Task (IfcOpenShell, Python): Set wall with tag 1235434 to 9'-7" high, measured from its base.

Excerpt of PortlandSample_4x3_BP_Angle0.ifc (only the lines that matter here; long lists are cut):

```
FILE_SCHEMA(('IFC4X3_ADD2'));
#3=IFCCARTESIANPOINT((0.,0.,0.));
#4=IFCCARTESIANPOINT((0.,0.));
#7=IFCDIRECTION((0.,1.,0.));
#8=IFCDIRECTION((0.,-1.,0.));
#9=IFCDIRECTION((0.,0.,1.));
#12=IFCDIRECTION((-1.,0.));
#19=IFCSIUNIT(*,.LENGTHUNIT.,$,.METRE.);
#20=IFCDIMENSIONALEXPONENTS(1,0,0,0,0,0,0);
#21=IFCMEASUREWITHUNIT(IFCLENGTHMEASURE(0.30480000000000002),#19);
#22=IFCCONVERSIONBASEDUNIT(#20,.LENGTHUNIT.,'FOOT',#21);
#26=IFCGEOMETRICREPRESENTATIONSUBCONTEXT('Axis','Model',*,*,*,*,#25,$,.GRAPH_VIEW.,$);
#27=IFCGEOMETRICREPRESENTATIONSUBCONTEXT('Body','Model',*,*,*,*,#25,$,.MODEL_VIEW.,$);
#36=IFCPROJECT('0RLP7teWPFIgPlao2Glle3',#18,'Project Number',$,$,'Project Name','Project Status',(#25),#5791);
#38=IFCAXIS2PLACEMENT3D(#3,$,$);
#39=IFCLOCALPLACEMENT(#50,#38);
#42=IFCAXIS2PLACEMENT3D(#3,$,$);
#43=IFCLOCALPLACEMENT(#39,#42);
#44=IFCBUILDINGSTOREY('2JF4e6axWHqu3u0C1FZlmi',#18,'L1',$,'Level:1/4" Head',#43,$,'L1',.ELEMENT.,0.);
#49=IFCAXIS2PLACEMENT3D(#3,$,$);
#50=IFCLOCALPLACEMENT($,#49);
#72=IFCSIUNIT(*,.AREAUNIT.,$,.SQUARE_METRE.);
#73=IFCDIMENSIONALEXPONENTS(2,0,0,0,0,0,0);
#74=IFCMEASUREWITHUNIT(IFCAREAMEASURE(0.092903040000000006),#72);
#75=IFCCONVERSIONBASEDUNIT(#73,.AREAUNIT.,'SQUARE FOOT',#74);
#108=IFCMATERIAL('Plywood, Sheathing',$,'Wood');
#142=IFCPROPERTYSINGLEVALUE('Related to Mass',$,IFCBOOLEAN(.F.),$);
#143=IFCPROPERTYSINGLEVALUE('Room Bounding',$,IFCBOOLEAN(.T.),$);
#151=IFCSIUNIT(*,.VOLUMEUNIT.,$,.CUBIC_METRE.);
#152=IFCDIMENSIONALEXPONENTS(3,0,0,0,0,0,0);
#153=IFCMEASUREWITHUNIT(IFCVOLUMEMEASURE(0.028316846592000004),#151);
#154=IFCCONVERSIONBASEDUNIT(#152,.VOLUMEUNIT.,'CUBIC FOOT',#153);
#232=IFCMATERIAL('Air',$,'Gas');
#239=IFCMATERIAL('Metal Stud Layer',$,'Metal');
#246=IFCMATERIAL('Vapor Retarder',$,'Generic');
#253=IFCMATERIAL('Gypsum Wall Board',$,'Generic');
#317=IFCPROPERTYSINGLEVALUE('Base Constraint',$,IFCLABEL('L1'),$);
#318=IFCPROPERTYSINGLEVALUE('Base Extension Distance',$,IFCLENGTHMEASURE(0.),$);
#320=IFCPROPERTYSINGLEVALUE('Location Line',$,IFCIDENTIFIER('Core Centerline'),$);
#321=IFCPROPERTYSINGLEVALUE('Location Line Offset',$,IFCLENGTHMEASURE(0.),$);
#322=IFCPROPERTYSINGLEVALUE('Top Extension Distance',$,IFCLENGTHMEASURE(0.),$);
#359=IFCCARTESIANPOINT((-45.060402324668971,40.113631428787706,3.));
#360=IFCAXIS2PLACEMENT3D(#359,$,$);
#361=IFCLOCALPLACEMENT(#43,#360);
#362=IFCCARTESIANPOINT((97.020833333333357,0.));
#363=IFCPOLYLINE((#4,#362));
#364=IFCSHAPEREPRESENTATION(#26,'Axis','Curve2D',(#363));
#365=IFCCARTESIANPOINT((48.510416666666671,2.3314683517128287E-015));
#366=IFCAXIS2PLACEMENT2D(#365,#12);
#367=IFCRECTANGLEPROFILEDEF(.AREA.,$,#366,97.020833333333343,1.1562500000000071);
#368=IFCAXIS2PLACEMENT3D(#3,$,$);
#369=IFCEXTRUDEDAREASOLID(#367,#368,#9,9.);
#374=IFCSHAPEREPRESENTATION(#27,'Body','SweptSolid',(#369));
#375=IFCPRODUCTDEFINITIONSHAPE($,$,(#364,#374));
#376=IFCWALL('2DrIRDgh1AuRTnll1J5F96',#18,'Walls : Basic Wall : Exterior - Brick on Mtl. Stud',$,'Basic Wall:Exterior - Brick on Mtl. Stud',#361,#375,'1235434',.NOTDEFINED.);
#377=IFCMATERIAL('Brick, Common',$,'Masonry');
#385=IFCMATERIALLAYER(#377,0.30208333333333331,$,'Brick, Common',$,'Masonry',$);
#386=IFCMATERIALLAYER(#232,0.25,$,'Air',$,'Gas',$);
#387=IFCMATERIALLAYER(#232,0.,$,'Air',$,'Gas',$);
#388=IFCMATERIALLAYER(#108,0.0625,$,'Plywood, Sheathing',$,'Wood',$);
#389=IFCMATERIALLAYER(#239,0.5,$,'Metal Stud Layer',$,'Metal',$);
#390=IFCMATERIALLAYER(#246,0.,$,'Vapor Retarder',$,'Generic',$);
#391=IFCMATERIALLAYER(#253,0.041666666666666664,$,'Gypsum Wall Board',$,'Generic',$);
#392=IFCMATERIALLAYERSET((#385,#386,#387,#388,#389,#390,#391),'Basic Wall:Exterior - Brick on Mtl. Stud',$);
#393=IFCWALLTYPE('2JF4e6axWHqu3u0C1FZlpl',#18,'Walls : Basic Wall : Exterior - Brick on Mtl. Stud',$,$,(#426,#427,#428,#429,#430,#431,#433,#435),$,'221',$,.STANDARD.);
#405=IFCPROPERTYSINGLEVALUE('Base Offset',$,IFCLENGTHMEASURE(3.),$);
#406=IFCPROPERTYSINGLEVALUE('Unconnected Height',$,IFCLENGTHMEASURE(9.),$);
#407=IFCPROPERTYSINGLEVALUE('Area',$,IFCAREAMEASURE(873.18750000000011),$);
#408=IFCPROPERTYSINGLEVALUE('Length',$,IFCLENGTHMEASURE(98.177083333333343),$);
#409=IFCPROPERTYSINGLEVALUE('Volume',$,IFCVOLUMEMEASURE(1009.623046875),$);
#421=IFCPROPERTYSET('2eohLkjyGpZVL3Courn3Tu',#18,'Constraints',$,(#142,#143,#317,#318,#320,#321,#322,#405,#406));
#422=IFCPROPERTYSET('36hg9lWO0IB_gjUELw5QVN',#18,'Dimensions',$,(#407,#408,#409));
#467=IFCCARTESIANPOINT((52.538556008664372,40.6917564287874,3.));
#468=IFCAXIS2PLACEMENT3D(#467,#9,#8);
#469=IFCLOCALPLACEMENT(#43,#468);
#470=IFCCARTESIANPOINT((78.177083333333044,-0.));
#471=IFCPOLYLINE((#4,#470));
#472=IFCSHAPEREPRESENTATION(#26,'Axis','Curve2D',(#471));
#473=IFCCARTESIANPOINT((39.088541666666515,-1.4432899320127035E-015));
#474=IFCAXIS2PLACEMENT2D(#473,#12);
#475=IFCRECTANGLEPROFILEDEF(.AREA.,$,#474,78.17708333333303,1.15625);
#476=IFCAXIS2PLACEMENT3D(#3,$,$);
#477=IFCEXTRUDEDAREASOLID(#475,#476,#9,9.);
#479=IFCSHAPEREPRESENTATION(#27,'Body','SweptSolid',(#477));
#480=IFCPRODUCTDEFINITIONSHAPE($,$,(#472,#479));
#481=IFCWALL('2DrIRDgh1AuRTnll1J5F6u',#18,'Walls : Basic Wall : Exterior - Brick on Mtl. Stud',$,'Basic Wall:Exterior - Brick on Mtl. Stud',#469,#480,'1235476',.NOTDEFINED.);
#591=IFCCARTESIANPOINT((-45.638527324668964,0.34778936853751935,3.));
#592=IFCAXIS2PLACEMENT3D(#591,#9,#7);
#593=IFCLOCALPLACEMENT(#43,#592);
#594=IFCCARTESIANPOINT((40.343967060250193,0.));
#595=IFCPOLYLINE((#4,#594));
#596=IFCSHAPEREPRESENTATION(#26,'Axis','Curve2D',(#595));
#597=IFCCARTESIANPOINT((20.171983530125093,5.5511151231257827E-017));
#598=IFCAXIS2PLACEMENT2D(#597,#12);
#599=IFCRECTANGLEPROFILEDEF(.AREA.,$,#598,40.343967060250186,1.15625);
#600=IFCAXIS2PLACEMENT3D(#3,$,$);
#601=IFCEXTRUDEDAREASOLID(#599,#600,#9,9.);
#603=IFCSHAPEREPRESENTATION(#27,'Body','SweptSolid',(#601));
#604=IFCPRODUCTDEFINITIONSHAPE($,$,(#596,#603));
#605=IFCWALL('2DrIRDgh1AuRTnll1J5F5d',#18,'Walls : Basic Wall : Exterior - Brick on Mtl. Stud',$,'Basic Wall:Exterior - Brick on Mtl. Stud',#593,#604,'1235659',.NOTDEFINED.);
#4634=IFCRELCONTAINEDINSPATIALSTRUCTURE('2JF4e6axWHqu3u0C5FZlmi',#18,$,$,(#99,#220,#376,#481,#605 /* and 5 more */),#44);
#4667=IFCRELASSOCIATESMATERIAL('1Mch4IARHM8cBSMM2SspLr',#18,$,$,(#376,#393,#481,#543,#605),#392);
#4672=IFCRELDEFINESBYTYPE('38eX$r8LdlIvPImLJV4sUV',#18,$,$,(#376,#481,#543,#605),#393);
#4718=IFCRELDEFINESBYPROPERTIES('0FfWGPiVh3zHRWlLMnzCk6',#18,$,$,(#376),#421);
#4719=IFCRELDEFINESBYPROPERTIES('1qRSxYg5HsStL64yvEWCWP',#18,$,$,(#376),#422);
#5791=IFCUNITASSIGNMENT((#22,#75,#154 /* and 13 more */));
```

```python
import ifcopenshell
import ifcopenshell.api.pset
import ifcopenshell.geom
import ifcopenshell.util.element
import ifcopenshell.util.representation
import ifcopenshell.util.shape
import ifcopenshell.util.unit

model = ifcopenshell.open("PortlandSample_4x3_BP_Angle0.ifc")
unit_scale = ifcopenshell.util.unit.calculate_unit_scale(model)
area_scale = ifcopenshell.util.unit.calculate_unit_scale(model, "AREAUNIT")
volume_scale = ifcopenshell.util.unit.calculate_unit_scale(model, "VOLUMEUNIT")
settings = ifcopenshell.geom.settings()


def volume(element):
    """Net volume in cubic metres, openings subtracted."""
    shape = ifcopenshell.geom.create_shape(settings, element)
    return ifcopenshell.util.shape.get_volume(shape.geometry)


wall = model.by_guid("2DrIRDgh1AuRTnll1J5F96")
before = volume(wall)

body = ifcopenshell.util.representation.get_representation(wall, "Model", "Body")
solid = body.Items[0]
old_height = solid.Depth
solid.Depth = 115 * 0.0254 / unit_scale
after = volume(wall)
thickness = 0.3524  # wall thickness in metres

# Update the stored height, areas and volumes.
pset = model.by_id(ifcopenshell.util.element.get_pset(wall, "Constraints", should_inherit=False)["id"])
ifcopenshell.api.pset.edit_pset(model, pset=pset, properties={
    "Unconnected Height": model.create_entity("IfcLengthMeasure", solid.Depth),
})
pset = model.by_id(ifcopenshell.util.element.get_pset(wall, "Dimensions", should_inherit=False)["id"])
ifcopenshell.api.pset.edit_pset(model, pset=pset, properties={
    "Area": model.create_entity("IfcAreaMeasure", after / thickness / area_scale),
    "Volume": model.create_entity("IfcVolumeMeasure", after / volume_scale),
})

print(f"height {old_height:g} -> {solid.Depth:g}, volume {before:.3f} -> {after:.3f} m3")

model.write("PortlandSample_4x3_BP_Angle0_updated.ifc")
```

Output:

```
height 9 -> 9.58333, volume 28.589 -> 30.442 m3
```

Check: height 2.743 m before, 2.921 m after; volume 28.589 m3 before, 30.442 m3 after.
